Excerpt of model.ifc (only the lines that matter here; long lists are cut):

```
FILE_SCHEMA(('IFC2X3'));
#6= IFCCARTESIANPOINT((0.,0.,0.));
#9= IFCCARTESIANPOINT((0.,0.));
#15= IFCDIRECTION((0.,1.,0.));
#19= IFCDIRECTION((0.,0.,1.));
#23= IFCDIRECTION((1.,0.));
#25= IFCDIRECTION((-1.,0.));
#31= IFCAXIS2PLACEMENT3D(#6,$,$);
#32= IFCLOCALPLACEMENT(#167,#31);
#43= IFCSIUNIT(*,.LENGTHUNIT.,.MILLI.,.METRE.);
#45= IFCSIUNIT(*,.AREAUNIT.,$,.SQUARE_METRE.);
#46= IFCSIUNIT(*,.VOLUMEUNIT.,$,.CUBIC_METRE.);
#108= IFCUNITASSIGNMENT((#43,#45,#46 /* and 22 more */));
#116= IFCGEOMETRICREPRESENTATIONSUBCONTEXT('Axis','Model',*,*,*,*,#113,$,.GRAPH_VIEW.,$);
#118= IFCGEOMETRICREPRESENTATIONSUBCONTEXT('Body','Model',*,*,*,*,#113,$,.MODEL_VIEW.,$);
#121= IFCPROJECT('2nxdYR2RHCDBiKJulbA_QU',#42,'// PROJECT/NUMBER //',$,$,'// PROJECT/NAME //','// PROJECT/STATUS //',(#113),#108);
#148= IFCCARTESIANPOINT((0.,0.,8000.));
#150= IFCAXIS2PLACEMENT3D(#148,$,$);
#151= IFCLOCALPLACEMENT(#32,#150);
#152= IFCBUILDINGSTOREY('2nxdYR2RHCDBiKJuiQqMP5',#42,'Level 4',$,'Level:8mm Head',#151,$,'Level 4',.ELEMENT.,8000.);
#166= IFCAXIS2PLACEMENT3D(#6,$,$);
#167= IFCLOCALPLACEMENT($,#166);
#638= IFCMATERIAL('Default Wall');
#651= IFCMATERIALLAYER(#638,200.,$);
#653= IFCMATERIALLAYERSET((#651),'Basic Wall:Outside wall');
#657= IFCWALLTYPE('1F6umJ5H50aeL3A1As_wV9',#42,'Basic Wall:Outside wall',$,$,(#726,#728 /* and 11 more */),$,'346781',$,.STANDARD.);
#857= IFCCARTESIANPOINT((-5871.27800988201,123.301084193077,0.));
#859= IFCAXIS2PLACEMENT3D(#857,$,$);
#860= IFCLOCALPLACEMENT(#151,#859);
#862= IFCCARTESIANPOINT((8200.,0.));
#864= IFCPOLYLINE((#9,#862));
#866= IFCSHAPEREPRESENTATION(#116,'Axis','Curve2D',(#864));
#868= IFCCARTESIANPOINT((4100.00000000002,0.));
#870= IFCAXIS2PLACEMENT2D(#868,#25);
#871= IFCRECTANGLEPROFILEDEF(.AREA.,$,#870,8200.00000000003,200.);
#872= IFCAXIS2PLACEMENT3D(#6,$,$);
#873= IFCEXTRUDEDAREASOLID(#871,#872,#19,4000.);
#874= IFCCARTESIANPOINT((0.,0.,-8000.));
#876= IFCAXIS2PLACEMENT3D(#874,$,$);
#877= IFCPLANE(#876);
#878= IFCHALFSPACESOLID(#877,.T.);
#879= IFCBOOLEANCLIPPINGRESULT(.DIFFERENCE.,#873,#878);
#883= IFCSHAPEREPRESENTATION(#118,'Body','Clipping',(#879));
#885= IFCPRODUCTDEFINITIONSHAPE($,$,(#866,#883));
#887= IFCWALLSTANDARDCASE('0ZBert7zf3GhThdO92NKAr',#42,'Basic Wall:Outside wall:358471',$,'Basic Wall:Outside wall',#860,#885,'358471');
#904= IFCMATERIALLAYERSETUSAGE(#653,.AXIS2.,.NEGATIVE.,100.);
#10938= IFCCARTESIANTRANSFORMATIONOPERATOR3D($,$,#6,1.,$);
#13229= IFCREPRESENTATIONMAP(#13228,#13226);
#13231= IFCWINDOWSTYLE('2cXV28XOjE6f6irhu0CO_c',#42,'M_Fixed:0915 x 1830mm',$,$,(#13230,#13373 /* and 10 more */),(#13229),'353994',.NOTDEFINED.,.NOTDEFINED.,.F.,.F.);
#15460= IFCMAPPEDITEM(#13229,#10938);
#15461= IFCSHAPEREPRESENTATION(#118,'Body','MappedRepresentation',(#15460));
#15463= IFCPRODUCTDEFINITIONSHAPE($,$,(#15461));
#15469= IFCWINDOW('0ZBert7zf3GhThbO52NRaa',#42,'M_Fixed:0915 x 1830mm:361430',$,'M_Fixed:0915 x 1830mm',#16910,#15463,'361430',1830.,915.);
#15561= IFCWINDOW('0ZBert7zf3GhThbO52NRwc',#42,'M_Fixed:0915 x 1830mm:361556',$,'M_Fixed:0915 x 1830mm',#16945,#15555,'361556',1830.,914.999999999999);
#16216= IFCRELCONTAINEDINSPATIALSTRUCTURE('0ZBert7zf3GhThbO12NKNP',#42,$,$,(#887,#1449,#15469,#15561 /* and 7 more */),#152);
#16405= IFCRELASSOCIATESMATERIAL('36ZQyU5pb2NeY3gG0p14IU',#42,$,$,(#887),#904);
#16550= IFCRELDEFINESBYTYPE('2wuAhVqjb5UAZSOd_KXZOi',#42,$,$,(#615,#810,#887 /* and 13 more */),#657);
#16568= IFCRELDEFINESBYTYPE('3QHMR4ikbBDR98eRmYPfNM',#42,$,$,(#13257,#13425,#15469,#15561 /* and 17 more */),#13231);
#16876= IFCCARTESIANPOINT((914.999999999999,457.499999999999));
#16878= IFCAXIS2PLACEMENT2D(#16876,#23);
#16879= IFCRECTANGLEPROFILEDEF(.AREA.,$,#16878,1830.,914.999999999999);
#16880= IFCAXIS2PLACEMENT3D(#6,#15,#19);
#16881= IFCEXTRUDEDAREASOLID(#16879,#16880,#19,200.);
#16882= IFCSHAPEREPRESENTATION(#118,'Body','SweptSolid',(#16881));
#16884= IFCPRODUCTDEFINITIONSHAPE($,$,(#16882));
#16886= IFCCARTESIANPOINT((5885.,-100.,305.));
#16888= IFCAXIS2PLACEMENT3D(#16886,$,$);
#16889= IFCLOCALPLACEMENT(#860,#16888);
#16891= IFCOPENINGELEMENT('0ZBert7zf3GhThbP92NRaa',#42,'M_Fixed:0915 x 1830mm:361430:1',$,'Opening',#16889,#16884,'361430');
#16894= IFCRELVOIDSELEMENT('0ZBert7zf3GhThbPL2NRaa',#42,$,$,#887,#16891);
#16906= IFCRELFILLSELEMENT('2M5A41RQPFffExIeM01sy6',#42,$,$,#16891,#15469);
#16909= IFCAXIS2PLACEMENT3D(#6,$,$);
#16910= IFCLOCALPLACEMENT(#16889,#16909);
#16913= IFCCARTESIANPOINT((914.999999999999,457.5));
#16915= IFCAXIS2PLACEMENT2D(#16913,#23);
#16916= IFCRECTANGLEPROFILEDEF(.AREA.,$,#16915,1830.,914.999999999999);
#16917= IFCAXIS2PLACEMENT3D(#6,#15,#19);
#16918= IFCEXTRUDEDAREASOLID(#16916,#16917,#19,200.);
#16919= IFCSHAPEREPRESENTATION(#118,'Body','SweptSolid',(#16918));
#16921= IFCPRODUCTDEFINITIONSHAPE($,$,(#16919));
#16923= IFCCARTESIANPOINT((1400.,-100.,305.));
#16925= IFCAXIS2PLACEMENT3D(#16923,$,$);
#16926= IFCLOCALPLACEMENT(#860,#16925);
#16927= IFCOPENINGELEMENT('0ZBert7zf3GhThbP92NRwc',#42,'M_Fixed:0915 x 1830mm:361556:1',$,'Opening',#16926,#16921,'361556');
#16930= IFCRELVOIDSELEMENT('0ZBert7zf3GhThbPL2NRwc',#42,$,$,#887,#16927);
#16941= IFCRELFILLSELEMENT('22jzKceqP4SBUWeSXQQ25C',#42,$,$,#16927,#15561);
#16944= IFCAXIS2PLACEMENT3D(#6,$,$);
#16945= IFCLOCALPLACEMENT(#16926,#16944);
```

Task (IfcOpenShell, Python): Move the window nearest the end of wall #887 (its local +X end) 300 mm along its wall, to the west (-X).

```python
import ifcopenshell
import ifcopenshell.api.geometry
import ifcopenshell.util.placement

model = ifcopenshell.open("model.ifc")

window = model.by_guid("0ZBert7zf3GhThbO52NRaa")
opening = window.FillsVoids[0].RelatingOpeningElement
wall = opening.VoidsElements[0].RelatingBuildingElement

wall_matrix = ifcopenshell.util.placement.get_local_placement(wall.ObjectPlacement)
shift = wall_matrix[:3, 0] * -300.0
before = ifcopenshell.util.placement.get_local_placement(window.ObjectPlacement)[:3, 3].copy()

# The window is placed relative to its opening, so it follows when the opening moves.
matrix = ifcopenshell.util.placement.get_local_placement(opening.ObjectPlacement)
matrix[:3, 3] += shift
ifcopenshell.api.geometry.edit_object_placement(
    model, product=opening, matrix=matrix, is_si=False, should_transform_children=True
)

after = ifcopenshell.util.placement.get_local_placement(window.ObjectPlacement)[:3, 3]
print("window moved by", (after - before).round(3) + 0.0)

model.write("model_v2.ifc")
```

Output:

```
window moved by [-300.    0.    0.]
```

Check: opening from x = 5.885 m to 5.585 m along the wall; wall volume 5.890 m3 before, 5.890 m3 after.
